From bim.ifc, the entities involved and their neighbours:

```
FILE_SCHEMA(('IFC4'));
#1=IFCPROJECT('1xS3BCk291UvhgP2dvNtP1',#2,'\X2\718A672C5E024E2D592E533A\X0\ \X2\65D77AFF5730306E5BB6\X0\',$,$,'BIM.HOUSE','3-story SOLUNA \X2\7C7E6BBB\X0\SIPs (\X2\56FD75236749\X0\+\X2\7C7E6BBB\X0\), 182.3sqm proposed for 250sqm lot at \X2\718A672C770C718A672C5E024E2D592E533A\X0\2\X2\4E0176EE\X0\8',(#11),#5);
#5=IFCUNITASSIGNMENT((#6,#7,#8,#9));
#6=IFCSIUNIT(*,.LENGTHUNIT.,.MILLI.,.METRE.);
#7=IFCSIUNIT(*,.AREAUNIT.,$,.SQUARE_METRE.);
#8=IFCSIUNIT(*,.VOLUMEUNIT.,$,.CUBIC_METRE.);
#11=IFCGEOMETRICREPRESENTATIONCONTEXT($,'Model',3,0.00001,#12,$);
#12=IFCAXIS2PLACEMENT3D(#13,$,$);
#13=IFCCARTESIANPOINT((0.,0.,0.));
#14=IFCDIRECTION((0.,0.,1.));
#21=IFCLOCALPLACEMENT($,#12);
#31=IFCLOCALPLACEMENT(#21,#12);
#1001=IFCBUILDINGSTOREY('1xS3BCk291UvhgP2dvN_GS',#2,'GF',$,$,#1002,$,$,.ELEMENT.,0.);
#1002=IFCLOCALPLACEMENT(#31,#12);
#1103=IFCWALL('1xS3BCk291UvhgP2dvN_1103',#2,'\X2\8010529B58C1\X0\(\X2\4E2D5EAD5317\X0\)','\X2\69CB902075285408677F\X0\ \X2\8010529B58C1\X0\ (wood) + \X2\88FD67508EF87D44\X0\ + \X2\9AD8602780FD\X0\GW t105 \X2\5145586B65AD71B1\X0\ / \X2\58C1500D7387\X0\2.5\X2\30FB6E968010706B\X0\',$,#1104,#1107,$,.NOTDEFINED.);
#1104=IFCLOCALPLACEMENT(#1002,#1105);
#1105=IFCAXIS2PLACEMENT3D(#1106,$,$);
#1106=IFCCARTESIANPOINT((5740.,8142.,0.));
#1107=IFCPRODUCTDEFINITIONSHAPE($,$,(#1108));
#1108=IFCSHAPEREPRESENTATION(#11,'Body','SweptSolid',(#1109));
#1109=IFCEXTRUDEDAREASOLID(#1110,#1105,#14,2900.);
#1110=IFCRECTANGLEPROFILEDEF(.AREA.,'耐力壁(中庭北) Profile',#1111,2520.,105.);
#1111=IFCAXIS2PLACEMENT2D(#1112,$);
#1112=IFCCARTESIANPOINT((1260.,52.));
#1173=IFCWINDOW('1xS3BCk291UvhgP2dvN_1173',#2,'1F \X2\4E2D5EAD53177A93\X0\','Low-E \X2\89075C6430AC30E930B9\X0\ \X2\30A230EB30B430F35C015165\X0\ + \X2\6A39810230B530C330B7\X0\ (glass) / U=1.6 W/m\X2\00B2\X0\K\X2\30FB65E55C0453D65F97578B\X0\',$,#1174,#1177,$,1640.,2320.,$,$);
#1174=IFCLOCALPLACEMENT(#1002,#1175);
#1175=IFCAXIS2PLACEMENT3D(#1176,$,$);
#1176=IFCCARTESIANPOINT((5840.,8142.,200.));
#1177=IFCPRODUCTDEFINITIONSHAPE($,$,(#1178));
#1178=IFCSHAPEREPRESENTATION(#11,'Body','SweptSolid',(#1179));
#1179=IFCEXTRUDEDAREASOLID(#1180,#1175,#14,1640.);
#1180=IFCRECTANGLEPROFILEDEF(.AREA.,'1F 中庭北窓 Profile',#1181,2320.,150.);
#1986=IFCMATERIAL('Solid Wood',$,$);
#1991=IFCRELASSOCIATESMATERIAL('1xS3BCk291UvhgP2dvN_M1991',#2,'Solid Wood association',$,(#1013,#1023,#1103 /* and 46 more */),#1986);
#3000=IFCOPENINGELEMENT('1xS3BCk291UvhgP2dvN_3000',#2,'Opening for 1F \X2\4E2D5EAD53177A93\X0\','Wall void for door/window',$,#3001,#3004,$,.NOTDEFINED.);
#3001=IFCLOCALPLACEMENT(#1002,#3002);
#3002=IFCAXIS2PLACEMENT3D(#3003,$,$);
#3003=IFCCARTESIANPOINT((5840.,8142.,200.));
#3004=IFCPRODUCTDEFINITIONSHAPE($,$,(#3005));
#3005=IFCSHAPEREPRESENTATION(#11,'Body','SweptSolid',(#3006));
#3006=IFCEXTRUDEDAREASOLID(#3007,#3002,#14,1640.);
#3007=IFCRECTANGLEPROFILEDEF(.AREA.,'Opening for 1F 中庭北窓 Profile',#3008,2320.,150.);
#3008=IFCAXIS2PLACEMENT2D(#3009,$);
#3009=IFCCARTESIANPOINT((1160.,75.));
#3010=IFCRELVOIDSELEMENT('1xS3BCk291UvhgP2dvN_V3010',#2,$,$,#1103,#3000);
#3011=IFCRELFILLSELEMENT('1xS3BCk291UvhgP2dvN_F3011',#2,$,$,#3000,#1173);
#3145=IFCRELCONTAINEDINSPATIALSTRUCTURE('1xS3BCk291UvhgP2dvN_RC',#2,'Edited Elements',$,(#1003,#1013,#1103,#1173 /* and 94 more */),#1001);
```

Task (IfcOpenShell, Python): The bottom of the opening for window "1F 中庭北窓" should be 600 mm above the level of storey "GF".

```python
import numpy as np
import ifcopenshell
import ifcopenshell.api.geometry
import ifcopenshell.geom
import ifcopenshell.util.element
import ifcopenshell.util.placement
import ifcopenshell.util.shape
import ifcopenshell.util.unit

model = ifcopenshell.open("bim.ifc")
unit_scale = ifcopenshell.util.unit.calculate_unit_scale(model)

window = model.by_id(1173)
opening = window.FillsVoids[0].RelatingOpeningElement
storey = ifcopenshell.util.element.get_container(window, ifc_class="IfcBuildingStorey")
level = ifcopenshell.util.placement.get_local_placement(storey.ObjectPlacement)[2, 3]

# The opening's origin need not be at the sill, so measure its lowest point.
shape = ifcopenshell.geom.create_shape(ifcopenshell.geom.settings(), opening)
bottom = ifcopenshell.util.shape.get_shape_bottom_elevation(shape, shape.geometry) / unit_scale
dz = level + 0.6 / unit_scale - bottom

shift = np.array([0.0, 0.0, dz])
# The window is not placed relative to its opening, so move both.
for product in (opening, window):
    matrix = ifcopenshell.util.placement.get_local_placement(product.ObjectPlacement)
    matrix[:3, 3] += shift
    ifcopenshell.api.geometry.edit_object_placement(model, product=product, matrix=matrix, is_si=False)

print(f"moved by {dz * unit_scale:+.3f} m")

model.write("bim_v2.ifc")
```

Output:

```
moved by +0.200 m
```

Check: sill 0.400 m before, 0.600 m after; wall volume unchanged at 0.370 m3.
